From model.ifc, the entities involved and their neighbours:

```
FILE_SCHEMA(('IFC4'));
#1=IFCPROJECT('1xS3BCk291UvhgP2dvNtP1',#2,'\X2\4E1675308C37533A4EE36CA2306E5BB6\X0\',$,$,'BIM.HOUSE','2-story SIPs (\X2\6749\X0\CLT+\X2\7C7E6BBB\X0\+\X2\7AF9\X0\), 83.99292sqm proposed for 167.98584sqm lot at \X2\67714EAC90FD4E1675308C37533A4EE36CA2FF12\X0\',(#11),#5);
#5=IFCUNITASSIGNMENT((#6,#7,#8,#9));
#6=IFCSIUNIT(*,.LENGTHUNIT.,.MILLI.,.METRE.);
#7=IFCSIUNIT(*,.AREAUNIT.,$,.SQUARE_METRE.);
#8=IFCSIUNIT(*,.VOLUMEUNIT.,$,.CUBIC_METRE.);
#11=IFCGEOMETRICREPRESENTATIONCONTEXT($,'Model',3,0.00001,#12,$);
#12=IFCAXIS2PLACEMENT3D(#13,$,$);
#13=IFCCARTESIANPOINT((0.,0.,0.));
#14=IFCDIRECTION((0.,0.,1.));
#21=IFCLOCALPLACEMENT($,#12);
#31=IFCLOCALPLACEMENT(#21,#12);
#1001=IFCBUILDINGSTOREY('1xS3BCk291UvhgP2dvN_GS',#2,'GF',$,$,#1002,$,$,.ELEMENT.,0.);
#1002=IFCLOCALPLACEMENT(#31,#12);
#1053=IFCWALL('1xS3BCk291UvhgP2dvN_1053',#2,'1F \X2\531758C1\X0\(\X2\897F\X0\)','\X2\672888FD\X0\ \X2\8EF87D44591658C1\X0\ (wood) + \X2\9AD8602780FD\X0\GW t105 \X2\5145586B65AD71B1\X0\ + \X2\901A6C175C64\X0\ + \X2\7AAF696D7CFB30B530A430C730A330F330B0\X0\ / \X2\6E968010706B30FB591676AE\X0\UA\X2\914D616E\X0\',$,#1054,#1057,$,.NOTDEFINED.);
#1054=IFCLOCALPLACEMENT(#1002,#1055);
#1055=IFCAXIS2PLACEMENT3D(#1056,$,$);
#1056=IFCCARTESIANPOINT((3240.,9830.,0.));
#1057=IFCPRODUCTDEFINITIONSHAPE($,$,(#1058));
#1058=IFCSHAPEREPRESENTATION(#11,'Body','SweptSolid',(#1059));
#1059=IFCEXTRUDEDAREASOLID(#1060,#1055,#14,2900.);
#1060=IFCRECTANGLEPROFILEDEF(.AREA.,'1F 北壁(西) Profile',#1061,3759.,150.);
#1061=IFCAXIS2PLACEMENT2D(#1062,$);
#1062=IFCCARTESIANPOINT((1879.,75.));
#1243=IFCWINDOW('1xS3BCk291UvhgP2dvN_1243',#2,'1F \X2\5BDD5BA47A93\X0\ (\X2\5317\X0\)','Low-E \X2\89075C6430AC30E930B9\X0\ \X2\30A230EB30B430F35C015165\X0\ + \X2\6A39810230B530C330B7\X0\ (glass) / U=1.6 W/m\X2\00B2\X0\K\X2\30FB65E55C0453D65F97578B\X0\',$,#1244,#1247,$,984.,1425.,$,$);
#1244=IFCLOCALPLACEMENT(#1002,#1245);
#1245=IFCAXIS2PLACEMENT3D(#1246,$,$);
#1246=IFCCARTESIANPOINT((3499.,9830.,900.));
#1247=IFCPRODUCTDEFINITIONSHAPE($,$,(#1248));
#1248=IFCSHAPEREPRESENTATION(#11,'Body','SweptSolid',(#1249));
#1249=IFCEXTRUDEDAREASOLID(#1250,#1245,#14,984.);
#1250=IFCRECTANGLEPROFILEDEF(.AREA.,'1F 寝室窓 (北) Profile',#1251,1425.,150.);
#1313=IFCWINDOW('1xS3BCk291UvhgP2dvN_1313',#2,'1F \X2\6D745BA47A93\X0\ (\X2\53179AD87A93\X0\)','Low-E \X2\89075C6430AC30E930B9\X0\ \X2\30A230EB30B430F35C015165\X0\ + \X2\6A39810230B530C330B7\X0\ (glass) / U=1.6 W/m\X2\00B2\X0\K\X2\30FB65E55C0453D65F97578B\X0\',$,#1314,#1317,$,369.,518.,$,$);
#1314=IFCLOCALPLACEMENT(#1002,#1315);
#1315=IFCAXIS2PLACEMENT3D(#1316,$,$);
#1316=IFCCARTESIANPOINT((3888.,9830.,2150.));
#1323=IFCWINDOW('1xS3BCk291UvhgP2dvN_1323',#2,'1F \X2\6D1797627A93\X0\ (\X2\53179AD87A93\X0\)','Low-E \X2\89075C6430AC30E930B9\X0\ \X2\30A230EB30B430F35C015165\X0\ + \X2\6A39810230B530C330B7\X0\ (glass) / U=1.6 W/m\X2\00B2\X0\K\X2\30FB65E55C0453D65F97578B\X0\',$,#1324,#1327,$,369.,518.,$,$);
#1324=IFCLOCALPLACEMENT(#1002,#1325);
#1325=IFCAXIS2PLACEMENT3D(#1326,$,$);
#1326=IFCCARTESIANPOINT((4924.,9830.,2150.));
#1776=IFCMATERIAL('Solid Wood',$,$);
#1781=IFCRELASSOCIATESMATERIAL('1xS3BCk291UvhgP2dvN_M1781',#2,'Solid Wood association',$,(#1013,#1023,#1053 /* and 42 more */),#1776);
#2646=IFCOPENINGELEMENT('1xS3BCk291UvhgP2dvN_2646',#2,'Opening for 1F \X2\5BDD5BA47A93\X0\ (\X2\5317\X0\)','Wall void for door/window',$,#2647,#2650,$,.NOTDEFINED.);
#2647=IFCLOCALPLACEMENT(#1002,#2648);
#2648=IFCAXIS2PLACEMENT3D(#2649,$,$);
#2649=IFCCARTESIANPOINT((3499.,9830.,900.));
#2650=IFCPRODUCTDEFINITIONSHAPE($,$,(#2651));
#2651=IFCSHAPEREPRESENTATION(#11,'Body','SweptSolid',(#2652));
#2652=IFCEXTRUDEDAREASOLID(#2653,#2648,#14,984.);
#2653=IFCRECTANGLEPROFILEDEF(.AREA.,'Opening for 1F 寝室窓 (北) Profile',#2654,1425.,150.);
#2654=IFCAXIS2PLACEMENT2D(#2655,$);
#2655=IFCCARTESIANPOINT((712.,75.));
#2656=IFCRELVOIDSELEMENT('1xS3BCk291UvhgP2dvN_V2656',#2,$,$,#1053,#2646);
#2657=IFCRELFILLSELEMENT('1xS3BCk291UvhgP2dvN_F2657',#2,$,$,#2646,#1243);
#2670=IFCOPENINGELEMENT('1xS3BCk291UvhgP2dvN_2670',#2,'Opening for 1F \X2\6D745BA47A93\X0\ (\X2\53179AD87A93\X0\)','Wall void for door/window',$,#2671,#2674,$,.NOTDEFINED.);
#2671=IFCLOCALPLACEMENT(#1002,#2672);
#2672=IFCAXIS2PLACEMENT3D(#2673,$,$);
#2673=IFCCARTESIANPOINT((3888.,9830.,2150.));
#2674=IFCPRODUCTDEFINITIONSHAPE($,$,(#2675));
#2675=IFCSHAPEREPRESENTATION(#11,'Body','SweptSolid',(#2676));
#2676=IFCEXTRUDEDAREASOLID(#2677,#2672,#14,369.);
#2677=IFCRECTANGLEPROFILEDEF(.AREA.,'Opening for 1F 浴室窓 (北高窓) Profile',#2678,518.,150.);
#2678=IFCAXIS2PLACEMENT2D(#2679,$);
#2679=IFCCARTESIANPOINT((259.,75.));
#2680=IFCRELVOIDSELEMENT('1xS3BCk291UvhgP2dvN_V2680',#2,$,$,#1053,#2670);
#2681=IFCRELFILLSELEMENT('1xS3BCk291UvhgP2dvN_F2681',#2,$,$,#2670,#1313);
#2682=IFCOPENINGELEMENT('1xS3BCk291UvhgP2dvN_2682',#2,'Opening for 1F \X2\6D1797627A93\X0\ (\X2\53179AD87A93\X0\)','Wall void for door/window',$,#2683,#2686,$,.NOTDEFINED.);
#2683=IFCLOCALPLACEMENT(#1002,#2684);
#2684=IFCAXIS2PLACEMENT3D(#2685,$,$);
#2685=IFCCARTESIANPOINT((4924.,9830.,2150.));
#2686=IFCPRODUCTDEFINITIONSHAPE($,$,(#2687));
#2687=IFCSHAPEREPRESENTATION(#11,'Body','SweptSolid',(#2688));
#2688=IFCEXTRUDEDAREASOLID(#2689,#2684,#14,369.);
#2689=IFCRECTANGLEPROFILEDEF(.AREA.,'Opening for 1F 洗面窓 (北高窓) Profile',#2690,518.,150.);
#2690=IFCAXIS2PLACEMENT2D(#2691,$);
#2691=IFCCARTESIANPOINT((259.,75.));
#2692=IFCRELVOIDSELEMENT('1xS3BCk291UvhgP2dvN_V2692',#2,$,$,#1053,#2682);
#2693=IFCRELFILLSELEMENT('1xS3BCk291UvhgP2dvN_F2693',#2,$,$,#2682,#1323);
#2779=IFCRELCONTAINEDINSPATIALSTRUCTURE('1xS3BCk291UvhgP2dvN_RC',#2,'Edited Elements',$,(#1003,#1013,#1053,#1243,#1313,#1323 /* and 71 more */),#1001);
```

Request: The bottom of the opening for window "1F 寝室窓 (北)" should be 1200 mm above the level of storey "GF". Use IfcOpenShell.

```python
import numpy as np
import ifcopenshell
import ifcopenshell.api.geometry
import ifcopenshell.geom
import ifcopenshell.util.element
import ifcopenshell.util.placement
import ifcopenshell.util.shape
import ifcopenshell.util.unit

model = ifcopenshell.open("model.ifc")
unit_scale = ifcopenshell.util.unit.calculate_unit_scale(model)

window = model.by_guid("1xS3BCk291UvhgP2dvN_1243")
opening = window.FillsVoids[0].RelatingOpeningElement
storey = ifcopenshell.util.element.get_container(window, ifc_class="IfcBuildingStorey")
level = ifcopenshell.util.placement.get_local_placement(storey.ObjectPlacement)[2, 3]

# The opening's origin need not be at the sill, so measure its lowest point.
shape = ifcopenshell.geom.create_shape(ifcopenshell.geom.settings(), opening)
bottom = ifcopenshell.util.shape.get_shape_bottom_elevation(shape, shape.geometry) / unit_scale
dz = level + 1200.0 - bottom

shift = np.array([0.0, 0.0, dz])
# The window is not placed relative to its opening, so move both.
for product in (opening, window):
    matrix = ifcopenshell.util.placement.get_local_placement(product.ObjectPlacement)
    matrix[:3, 3] += shift
    ifcopenshell.api.geometry.edit_object_placement(model, product=product, matrix=matrix, is_si=False)

print(f"moved by {dz * unit_scale:+.3f} m")

model.write("model_rev.ifc")
```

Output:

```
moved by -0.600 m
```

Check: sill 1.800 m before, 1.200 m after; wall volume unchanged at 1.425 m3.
